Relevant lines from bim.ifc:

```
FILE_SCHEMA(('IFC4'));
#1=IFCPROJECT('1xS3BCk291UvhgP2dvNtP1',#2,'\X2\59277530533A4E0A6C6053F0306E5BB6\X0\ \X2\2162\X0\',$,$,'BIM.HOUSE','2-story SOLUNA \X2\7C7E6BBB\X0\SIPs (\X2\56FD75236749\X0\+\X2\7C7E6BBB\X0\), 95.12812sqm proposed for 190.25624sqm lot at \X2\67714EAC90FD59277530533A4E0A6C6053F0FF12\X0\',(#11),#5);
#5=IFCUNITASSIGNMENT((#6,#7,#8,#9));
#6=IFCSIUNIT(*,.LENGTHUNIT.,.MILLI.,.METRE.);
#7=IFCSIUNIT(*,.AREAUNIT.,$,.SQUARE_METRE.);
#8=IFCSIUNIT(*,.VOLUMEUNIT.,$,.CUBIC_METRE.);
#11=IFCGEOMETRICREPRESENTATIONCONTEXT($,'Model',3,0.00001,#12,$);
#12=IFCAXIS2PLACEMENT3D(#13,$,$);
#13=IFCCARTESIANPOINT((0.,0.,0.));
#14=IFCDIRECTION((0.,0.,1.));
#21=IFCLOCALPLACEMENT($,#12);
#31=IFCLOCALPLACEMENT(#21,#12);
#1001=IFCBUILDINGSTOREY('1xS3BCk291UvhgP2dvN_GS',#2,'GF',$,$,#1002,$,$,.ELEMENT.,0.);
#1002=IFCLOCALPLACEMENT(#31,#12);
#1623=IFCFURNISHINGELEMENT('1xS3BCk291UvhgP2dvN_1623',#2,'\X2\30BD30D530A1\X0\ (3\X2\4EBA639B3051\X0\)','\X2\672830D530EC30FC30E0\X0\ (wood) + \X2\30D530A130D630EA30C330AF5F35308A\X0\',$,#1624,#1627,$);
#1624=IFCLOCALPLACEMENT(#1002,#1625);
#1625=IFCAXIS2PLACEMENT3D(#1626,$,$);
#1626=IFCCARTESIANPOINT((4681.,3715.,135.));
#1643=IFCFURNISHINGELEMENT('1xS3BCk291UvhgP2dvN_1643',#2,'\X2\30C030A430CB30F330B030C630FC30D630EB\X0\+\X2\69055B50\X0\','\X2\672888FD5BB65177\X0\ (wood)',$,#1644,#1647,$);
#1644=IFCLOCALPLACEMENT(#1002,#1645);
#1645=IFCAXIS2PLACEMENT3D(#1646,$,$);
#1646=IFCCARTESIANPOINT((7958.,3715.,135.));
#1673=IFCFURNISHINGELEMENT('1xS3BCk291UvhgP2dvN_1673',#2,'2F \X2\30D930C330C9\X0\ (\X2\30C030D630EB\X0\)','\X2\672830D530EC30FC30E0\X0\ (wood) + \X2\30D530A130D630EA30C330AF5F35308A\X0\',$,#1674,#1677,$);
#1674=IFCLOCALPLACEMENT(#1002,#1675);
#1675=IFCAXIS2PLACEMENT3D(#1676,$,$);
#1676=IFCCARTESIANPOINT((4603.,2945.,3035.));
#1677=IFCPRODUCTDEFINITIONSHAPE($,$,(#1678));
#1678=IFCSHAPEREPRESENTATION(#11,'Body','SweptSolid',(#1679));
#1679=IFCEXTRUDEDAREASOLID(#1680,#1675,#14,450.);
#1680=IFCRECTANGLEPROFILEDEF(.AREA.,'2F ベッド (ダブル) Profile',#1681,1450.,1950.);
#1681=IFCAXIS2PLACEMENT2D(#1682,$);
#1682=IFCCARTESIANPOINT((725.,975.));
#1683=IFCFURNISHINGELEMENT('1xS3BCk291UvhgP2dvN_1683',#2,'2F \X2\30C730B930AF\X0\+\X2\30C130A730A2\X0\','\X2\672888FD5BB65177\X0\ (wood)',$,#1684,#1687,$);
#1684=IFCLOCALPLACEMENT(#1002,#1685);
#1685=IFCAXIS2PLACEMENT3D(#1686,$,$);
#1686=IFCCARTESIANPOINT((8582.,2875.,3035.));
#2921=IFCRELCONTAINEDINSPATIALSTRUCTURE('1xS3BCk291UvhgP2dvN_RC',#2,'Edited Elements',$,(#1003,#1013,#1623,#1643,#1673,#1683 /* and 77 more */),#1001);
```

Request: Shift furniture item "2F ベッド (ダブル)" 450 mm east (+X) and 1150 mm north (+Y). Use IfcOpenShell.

```python
import ifcopenshell
import ifcopenshell.api.geometry
import ifcopenshell.util.placement
import ifcopenshell.util.unit

model = ifcopenshell.open("bim.ifc")
unit_scale = ifcopenshell.util.unit.calculate_unit_scale(model)

item = model.by_id(1673)
matrix = ifcopenshell.util.placement.get_local_placement(item.ObjectPlacement)
matrix[0, 3] += 0.45 / unit_scale
matrix[1, 3] += 1.15 / unit_scale
ifcopenshell.api.geometry.edit_object_placement(model, product=item, matrix=matrix, is_si=False)

print(ifcopenshell.util.placement.get_local_placement(item.ObjectPlacement).round(3) + 0.0)

model.write("bim_edited.ifc")
```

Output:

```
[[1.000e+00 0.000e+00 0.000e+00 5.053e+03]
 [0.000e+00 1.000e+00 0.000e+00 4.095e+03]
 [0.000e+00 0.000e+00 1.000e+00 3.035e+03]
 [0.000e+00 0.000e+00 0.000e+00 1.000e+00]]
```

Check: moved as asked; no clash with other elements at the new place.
